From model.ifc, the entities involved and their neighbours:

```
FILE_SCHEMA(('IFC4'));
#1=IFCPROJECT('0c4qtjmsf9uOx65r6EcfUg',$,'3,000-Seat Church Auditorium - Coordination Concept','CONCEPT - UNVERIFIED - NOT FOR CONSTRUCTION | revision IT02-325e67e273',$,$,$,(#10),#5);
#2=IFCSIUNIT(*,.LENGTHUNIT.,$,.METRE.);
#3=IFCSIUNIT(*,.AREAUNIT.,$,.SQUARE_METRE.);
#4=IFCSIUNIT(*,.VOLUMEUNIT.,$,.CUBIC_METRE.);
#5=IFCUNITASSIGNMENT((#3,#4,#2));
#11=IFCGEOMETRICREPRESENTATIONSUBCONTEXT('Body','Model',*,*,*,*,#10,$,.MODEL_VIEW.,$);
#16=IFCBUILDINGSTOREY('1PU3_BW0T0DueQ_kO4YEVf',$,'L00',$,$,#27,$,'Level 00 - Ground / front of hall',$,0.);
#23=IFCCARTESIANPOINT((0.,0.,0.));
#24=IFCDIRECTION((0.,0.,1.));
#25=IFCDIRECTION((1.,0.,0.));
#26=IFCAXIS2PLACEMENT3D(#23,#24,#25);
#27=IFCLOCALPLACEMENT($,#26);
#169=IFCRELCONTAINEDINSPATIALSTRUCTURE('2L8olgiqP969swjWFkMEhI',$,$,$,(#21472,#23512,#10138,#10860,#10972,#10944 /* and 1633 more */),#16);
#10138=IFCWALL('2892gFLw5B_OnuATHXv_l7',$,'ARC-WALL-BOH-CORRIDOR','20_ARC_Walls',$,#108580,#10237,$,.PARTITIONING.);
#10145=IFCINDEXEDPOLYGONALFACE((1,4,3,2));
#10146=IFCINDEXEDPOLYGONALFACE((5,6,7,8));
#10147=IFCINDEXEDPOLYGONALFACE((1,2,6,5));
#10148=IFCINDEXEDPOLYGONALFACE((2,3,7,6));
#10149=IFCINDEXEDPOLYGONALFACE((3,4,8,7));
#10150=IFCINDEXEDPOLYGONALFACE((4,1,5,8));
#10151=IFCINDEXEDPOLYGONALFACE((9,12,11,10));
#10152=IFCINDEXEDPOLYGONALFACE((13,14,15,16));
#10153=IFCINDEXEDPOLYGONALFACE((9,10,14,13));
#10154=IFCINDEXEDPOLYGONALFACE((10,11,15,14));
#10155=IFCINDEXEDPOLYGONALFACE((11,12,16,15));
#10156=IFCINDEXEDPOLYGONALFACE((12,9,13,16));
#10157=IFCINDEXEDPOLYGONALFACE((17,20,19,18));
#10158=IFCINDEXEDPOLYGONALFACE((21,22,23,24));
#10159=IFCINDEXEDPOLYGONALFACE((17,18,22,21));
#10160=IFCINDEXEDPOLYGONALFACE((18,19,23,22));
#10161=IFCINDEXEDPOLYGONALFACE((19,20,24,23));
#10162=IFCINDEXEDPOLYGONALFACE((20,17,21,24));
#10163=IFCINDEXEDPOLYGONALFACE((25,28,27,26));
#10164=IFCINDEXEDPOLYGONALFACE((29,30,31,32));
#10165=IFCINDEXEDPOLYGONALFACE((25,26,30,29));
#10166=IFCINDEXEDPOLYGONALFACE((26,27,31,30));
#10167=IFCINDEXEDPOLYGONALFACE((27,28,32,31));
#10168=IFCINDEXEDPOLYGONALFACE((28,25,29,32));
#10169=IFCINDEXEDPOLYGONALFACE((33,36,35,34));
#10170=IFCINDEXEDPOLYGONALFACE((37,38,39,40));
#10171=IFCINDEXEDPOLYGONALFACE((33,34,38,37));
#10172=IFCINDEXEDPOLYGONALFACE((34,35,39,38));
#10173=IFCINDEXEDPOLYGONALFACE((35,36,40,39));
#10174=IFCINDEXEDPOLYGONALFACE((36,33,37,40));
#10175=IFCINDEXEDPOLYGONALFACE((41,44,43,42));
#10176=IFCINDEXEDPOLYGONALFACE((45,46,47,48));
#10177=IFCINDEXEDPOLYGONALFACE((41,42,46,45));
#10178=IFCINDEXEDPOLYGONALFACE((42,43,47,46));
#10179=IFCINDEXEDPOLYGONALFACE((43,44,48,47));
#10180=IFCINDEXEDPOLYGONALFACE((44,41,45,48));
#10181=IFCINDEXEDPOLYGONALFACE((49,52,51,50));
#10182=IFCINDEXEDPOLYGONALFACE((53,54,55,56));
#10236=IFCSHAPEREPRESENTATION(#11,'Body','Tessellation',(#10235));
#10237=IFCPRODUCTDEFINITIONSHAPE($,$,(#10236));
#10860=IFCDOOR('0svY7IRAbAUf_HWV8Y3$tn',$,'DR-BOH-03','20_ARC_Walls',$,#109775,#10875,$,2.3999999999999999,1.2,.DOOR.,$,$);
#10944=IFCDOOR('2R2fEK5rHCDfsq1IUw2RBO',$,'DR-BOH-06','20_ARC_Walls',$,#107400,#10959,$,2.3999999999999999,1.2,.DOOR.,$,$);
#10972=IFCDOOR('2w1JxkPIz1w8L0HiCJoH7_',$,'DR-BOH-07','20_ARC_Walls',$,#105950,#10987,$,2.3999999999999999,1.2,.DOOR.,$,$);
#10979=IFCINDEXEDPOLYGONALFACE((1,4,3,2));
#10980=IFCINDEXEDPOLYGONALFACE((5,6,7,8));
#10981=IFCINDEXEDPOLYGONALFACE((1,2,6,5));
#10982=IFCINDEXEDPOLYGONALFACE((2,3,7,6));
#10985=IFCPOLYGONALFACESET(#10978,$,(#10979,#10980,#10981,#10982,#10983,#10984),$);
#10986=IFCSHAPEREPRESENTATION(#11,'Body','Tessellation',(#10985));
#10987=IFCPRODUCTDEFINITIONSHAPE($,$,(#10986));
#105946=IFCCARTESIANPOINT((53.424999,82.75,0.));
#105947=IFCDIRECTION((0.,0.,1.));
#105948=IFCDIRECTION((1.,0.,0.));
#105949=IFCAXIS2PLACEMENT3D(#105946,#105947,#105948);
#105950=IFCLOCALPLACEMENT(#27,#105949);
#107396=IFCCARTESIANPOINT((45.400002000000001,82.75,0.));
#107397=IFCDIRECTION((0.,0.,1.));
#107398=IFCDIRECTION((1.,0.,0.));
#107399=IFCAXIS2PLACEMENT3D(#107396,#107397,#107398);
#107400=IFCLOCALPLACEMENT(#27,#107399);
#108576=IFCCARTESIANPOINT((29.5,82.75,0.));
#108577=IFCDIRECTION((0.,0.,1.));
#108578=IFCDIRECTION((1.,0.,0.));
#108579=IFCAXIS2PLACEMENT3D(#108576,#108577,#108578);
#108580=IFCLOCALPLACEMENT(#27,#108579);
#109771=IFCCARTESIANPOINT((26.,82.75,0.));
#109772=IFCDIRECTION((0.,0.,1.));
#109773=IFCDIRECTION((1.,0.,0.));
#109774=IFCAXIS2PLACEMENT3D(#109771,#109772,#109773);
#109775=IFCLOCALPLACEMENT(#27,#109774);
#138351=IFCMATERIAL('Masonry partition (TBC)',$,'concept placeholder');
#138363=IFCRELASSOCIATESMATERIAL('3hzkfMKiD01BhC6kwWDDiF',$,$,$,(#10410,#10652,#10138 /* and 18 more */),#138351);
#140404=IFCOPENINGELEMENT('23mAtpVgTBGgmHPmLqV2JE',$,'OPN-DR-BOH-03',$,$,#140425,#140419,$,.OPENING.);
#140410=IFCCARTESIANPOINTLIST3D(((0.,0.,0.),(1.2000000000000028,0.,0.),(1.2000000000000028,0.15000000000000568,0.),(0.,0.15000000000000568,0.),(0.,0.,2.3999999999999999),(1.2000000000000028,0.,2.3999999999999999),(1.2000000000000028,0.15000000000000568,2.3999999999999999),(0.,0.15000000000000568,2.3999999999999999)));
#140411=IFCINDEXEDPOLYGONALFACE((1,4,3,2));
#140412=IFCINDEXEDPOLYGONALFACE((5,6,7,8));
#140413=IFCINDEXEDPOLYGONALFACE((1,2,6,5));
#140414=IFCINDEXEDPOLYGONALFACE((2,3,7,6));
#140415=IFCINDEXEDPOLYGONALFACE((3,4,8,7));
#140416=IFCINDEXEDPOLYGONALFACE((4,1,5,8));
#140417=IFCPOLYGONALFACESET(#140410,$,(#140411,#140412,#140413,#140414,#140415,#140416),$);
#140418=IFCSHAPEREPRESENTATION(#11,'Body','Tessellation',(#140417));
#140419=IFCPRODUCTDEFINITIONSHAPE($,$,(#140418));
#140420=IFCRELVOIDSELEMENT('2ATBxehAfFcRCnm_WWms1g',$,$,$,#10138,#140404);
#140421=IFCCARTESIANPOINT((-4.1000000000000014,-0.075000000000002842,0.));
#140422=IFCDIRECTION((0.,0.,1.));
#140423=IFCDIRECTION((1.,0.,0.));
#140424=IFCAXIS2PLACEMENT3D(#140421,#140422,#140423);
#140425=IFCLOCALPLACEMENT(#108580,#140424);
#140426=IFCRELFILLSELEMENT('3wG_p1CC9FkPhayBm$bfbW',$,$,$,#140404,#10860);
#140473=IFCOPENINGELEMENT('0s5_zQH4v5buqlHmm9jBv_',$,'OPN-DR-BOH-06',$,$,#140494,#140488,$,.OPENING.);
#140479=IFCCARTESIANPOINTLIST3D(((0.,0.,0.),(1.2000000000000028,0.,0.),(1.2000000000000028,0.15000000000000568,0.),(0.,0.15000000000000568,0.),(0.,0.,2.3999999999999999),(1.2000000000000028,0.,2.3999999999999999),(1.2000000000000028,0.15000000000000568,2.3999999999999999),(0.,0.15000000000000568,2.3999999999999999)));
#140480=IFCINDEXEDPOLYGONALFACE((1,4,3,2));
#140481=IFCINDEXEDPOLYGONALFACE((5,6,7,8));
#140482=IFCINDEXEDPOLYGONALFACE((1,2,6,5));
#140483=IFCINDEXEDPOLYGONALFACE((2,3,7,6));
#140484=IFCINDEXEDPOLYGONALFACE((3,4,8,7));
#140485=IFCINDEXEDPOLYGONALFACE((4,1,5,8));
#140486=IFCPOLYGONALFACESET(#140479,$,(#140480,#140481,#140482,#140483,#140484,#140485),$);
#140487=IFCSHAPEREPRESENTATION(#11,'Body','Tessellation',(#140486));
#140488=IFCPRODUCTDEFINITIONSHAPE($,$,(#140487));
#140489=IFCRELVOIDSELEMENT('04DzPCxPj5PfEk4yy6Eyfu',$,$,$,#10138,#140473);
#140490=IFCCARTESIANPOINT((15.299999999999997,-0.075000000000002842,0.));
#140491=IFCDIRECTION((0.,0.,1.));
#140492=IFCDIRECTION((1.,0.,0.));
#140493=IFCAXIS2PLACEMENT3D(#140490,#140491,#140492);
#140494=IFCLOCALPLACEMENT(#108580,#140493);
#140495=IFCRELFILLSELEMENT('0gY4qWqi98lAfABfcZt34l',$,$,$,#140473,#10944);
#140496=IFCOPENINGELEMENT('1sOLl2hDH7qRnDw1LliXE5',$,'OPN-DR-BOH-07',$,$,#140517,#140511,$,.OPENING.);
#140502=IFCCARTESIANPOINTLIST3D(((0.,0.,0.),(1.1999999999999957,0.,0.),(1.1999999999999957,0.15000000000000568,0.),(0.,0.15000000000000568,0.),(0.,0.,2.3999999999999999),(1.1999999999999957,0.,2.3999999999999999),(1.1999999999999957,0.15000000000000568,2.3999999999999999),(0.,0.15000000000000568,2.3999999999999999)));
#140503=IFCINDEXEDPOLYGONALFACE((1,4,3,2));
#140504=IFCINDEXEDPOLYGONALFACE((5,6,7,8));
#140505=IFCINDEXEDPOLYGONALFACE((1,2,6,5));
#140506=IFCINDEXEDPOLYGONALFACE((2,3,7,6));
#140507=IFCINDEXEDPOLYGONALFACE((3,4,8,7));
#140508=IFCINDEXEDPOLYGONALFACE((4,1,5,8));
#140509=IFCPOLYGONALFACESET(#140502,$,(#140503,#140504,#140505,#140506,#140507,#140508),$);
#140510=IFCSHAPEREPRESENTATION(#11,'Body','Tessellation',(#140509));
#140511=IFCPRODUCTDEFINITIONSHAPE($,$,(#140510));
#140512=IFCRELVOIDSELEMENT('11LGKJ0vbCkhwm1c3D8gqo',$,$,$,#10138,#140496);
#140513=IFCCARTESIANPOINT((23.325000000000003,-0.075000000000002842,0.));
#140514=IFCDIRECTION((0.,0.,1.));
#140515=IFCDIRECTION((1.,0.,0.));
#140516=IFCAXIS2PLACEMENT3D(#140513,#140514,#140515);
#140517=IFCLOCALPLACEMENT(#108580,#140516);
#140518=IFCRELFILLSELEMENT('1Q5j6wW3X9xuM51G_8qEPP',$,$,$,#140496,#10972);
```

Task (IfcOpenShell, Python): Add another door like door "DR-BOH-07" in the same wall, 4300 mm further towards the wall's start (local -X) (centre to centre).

```python
import ifcopenshell
import ifcopenshell.api.feature
import ifcopenshell.api.geometry
import ifcopenshell.api.root
import ifcopenshell.geom
import ifcopenshell.util.element
import ifcopenshell.util.placement
import ifcopenshell.util.shape
import ifcopenshell.util.unit

model = ifcopenshell.open("model.ifc")
unit_scale = ifcopenshell.util.unit.calculate_unit_scale(model)
settings = ifcopenshell.geom.settings()


def volume(element):
    """Net volume in cubic metres, openings subtracted."""
    shape = ifcopenshell.geom.create_shape(settings, element)
    return ifcopenshell.util.shape.get_volume(shape.geometry)


door = model.by_guid("2w1JxkPIz1w8L0HiCJoH7_")
opening = door.FillsVoids[0].RelatingOpeningElement
wall = opening.VoidsElements[0].RelatingBuildingElement
before = volume(wall)
shift = ifcopenshell.util.placement.get_local_placement(wall.ObjectPlacement)[:3, 0] * -4.3 / unit_scale

# copy_class copies the void relationship, type, container and properties, but no geometry.
new_opening = ifcopenshell.api.root.copy_class(model, product=opening)
new_opening.Representation = ifcopenshell.util.element.copy_deep(
    model, opening.Representation, exclude=["IfcGeometricRepresentationContext", "IfcRepresentationMap"]
)
new_door = ifcopenshell.api.root.copy_class(model, product=door)
new_door.Representation = ifcopenshell.util.element.copy_deep(
    model, door.Representation, exclude=["IfcGeometricRepresentationContext", "IfcRepresentationMap"]
)
ifcopenshell.api.feature.add_filling(model, opening=new_opening, element=new_door)

for old, new in ((opening, new_opening), (door, new_door)):
    matrix = ifcopenshell.util.placement.get_local_placement(old.ObjectPlacement)
    matrix[:3, 3] += shift
    ifcopenshell.api.geometry.edit_object_placement(model, product=new, matrix=matrix, is_si=False)

after = volume(wall)

print(f"wall volume {before:.3f} -> {after:.3f} m3")

model.write("model_v2.ifc")
```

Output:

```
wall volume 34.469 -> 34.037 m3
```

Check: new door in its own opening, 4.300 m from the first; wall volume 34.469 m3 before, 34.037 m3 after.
